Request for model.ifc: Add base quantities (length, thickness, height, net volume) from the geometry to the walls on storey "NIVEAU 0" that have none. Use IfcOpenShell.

First a look at what the model holds.

```python
import ifcopenshell
import ifcopenshell.util.element
import ifcopenshell.util.unit

model = ifcopenshell.open("model.ifc")
print(model.schema)
for unit_type in ("LENGTHUNIT", "AREAUNIT", "VOLUMEUNIT"):
    print(unit_type, ifcopenshell.util.unit.calculate_unit_scale(model, unit_type))
storey = next(s for s in model.by_type("IfcBuildingStorey") if s.Name == "NIVEAU 0")
walls = [e for e in ifcopenshell.util.element.get_decomposition(storey) if e.is_a("IfcWall")]
for e in sorted(walls, key=lambda e: e.id()):
    print(e.id(), e.is_a(), e.Name, list(ifcopenshell.util.element.get_psets(e, qtos_only=True)), sep=" | ")
```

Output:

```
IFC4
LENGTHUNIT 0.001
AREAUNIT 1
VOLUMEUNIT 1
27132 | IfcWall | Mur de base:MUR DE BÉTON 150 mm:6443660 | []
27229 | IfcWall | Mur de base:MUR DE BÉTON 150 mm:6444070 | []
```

```python
import ifcopenshell
import ifcopenshell.api.pset
import ifcopenshell.geom
import ifcopenshell.util.element
import ifcopenshell.util.shape
import ifcopenshell.util.unit

model = ifcopenshell.open("model.ifc")
unit_scale = ifcopenshell.util.unit.calculate_unit_scale(model)
volume_scale = ifcopenshell.util.unit.calculate_unit_scale(model, "VOLUMEUNIT")
settings = ifcopenshell.geom.settings()

storey = next(s for s in model.by_type("IfcBuildingStorey") if s.Name == "NIVEAU 0")
walls = [e for e in ifcopenshell.util.element.get_decomposition(storey) if e.is_a("IfcWall")]

for e in sorted(walls, key=lambda e: e.id()):
    if ifcopenshell.util.element.get_psets(e, qtos_only=True, should_inherit=False):
        continue
    # Geometry comes back in metres, in the element's own axes.
    shape = ifcopenshell.geom.create_shape(settings, e)
    values = {
        "Length": ifcopenshell.util.shape.get_x(shape.geometry) / unit_scale,
        "Width": ifcopenshell.util.shape.get_y(shape.geometry) / unit_scale,
        "Height": ifcopenshell.util.shape.get_z(shape.geometry) / unit_scale,
        "NetVolume": ifcopenshell.util.shape.get_volume(shape.geometry) / volume_scale,
    }
    qto = ifcopenshell.api.pset.add_qto(model, product=e, name="Qto_WallBaseQuantities")
    ifcopenshell.api.pset.edit_qto(model, qto=qto, properties=values)
    print(e.id(), {k: round(v, 3) for k, v in values.items()})

model.write("model_rev.ifc")
```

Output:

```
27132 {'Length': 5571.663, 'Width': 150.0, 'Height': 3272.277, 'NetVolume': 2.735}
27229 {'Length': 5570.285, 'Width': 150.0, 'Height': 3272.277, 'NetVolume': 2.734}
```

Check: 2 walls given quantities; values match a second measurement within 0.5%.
